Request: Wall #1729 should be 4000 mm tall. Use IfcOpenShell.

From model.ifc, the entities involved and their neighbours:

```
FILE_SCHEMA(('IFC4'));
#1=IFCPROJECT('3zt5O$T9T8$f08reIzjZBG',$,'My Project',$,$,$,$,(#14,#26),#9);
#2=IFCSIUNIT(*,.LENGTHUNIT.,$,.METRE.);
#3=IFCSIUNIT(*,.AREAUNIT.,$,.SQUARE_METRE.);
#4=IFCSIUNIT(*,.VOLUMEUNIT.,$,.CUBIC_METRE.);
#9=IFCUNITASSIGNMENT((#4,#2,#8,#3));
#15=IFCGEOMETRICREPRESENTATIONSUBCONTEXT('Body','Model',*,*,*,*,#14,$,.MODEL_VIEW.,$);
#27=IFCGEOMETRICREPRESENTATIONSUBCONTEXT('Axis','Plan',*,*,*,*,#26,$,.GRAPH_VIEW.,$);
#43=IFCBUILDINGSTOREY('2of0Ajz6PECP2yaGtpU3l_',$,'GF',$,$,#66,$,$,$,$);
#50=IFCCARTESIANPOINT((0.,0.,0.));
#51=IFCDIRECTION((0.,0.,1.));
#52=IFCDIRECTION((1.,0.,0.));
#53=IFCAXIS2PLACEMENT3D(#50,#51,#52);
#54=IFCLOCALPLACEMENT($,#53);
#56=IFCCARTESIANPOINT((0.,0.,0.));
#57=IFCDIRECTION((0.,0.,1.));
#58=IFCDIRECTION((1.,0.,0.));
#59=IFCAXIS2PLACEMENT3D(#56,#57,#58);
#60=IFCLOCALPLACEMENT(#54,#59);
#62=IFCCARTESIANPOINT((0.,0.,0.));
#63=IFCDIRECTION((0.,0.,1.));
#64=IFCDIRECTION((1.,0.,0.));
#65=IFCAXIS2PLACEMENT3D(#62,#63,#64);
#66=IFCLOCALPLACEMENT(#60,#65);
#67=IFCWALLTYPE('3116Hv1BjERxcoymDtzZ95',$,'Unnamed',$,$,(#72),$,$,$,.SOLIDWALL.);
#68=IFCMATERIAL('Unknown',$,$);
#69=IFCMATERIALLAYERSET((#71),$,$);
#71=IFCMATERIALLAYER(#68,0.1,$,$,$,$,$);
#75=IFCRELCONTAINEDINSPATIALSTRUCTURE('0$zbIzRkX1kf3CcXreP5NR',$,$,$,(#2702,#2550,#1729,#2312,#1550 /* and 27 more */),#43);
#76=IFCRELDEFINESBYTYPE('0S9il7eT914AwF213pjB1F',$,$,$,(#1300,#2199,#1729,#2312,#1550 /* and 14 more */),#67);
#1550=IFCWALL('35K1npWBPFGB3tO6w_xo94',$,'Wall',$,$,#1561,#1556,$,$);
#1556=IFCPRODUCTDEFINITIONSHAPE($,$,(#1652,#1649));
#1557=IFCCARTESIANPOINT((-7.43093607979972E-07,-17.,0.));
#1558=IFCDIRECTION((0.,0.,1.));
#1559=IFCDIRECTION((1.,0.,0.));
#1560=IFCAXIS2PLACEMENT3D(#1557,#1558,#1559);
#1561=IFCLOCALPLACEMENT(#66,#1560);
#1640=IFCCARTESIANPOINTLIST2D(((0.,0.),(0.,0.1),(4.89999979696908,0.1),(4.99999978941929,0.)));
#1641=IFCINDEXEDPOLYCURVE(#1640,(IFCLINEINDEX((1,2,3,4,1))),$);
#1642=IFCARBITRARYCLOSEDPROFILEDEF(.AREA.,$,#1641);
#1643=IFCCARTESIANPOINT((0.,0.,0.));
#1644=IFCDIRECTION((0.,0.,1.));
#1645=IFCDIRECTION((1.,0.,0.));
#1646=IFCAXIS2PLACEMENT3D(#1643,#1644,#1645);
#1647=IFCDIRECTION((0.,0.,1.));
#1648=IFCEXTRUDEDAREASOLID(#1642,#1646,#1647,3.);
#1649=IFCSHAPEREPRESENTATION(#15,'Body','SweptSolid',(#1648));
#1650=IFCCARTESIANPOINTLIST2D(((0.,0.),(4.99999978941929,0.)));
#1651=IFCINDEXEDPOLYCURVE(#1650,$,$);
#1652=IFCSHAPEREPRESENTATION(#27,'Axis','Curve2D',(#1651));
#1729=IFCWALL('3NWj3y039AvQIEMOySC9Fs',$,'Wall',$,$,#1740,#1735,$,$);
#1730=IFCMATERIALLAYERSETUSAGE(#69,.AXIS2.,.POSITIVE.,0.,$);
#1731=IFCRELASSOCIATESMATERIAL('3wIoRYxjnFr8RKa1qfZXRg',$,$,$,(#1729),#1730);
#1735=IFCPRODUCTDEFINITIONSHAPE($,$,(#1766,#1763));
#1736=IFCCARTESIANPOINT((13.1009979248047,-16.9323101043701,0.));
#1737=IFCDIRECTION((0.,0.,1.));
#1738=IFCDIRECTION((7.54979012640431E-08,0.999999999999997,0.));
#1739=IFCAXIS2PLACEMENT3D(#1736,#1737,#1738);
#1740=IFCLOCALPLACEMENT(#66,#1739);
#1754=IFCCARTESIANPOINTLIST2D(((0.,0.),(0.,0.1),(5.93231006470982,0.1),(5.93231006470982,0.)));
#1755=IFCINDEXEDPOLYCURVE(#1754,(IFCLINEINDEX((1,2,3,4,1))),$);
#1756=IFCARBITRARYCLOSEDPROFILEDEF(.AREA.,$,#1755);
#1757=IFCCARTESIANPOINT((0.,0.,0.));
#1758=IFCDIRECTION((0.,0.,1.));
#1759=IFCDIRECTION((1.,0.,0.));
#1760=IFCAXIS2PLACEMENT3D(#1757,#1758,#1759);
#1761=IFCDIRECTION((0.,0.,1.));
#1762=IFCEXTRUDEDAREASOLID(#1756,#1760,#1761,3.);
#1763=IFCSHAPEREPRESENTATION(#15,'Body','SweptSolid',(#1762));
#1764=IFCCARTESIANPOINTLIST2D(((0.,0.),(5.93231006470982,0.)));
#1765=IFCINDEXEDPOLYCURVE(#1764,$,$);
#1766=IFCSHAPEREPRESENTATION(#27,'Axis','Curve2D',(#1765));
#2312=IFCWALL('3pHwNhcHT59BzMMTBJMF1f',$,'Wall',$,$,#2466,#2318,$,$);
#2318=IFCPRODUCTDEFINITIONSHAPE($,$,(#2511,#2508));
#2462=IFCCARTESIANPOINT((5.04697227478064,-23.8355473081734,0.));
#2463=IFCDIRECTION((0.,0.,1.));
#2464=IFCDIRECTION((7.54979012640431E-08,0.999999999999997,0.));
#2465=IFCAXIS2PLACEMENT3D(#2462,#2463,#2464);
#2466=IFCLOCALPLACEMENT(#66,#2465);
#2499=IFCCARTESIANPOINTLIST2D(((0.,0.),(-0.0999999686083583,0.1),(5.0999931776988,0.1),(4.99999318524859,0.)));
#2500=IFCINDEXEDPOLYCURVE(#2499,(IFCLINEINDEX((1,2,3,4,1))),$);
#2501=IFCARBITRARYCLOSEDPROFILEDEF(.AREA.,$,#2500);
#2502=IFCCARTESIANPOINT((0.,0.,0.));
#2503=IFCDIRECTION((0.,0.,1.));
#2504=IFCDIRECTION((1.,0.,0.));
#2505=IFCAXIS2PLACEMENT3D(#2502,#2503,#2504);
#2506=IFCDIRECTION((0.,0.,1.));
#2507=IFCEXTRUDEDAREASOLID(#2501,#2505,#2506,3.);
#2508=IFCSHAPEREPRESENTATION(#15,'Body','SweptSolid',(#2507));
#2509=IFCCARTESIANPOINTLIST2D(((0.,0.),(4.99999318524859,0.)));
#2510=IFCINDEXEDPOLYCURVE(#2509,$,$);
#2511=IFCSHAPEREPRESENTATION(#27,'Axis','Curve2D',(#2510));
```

```python
import ifcopenshell
import ifcopenshell.geom
import ifcopenshell.util.representation
import ifcopenshell.util.shape
import ifcopenshell.util.unit

model = ifcopenshell.open("model.ifc")
unit_scale = ifcopenshell.util.unit.calculate_unit_scale(model)
settings = ifcopenshell.geom.settings()


def volume(element):
    """Net volume in cubic metres, openings subtracted."""
    shape = ifcopenshell.geom.create_shape(settings, element)
    return ifcopenshell.util.shape.get_volume(shape.geometry)


wall = model.by_guid("3NWj3y039AvQIEMOySC9Fs")
before = volume(wall)

body = ifcopenshell.util.representation.get_representation(wall, "Model", "Body")
solid = body.Items[0]
old_height = solid.Depth
solid.Depth = 4 / unit_scale
after = volume(wall)

print(f"height {old_height:g} -> {solid.Depth:g}, volume {before:.3f} -> {after:.3f} m3")

model.write("model_edited.ifc")
```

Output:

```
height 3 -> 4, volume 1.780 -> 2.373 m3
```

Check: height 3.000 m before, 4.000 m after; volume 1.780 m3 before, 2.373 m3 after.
